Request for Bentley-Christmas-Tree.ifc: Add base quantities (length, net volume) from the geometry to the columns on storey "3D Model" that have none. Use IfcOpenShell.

First a look at what the model holds.

```python
import ifcopenshell
import ifcopenshell.util.element
import ifcopenshell.util.unit

model = ifcopenshell.open("Bentley-Christmas-Tree.ifc")
print(model.schema)
for unit_type in ("LENGTHUNIT", "AREAUNIT", "VOLUMEUNIT"):
    print(unit_type, ifcopenshell.util.unit.calculate_unit_scale(model, unit_type))
storey = next(s for s in model.by_type("IfcBuildingStorey") if s.Name == "3D Model")
columns = [e for e in ifcopenshell.util.element.get_decomposition(storey) if e.is_a("IfcColumn")]
for e in sorted(columns, key=lambda e: e.id()):
    print(e.id(), e.is_a(), e.Name, list(ifcopenshell.util.element.get_psets(e, qtos_only=True)), sep=" | ")
```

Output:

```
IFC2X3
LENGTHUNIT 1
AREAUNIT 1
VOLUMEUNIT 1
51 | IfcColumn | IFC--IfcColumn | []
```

```python
import ifcopenshell
import ifcopenshell.api.pset
import ifcopenshell.geom
import ifcopenshell.util.element
import ifcopenshell.util.shape
import ifcopenshell.util.unit

model = ifcopenshell.open("Bentley-Christmas-Tree.ifc")
unit_scale = ifcopenshell.util.unit.calculate_unit_scale(model)
volume_scale = ifcopenshell.util.unit.calculate_unit_scale(model, "VOLUMEUNIT")
settings = ifcopenshell.geom.settings()

storey = next(s for s in model.by_type("IfcBuildingStorey") if s.Name == "3D Model")
columns = [e for e in ifcopenshell.util.element.get_decomposition(storey) if e.is_a("IfcColumn")]

for e in sorted(columns, key=lambda e: e.id()):
    if ifcopenshell.util.element.get_psets(e, qtos_only=True, should_inherit=False):
        continue
    # Geometry comes back in metres, in the element's own axes.
    shape = ifcopenshell.geom.create_shape(settings, e)
    values = {
        "Length": ifcopenshell.util.shape.get_z(shape.geometry) / unit_scale,
        "NetVolume": ifcopenshell.util.shape.get_volume(shape.geometry) / volume_scale,
    }
    qto = ifcopenshell.api.pset.add_qto(model, product=e, name="BaseQuantities")
    ifcopenshell.api.pset.edit_qto(model, qto=qto, properties=values)
    print(e.id(), {k: round(v, 3) for k, v in values.items()})

model.write("Bentley-Christmas-Tree_rev.ifc")
```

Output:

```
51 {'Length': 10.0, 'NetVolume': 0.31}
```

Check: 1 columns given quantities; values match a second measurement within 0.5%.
